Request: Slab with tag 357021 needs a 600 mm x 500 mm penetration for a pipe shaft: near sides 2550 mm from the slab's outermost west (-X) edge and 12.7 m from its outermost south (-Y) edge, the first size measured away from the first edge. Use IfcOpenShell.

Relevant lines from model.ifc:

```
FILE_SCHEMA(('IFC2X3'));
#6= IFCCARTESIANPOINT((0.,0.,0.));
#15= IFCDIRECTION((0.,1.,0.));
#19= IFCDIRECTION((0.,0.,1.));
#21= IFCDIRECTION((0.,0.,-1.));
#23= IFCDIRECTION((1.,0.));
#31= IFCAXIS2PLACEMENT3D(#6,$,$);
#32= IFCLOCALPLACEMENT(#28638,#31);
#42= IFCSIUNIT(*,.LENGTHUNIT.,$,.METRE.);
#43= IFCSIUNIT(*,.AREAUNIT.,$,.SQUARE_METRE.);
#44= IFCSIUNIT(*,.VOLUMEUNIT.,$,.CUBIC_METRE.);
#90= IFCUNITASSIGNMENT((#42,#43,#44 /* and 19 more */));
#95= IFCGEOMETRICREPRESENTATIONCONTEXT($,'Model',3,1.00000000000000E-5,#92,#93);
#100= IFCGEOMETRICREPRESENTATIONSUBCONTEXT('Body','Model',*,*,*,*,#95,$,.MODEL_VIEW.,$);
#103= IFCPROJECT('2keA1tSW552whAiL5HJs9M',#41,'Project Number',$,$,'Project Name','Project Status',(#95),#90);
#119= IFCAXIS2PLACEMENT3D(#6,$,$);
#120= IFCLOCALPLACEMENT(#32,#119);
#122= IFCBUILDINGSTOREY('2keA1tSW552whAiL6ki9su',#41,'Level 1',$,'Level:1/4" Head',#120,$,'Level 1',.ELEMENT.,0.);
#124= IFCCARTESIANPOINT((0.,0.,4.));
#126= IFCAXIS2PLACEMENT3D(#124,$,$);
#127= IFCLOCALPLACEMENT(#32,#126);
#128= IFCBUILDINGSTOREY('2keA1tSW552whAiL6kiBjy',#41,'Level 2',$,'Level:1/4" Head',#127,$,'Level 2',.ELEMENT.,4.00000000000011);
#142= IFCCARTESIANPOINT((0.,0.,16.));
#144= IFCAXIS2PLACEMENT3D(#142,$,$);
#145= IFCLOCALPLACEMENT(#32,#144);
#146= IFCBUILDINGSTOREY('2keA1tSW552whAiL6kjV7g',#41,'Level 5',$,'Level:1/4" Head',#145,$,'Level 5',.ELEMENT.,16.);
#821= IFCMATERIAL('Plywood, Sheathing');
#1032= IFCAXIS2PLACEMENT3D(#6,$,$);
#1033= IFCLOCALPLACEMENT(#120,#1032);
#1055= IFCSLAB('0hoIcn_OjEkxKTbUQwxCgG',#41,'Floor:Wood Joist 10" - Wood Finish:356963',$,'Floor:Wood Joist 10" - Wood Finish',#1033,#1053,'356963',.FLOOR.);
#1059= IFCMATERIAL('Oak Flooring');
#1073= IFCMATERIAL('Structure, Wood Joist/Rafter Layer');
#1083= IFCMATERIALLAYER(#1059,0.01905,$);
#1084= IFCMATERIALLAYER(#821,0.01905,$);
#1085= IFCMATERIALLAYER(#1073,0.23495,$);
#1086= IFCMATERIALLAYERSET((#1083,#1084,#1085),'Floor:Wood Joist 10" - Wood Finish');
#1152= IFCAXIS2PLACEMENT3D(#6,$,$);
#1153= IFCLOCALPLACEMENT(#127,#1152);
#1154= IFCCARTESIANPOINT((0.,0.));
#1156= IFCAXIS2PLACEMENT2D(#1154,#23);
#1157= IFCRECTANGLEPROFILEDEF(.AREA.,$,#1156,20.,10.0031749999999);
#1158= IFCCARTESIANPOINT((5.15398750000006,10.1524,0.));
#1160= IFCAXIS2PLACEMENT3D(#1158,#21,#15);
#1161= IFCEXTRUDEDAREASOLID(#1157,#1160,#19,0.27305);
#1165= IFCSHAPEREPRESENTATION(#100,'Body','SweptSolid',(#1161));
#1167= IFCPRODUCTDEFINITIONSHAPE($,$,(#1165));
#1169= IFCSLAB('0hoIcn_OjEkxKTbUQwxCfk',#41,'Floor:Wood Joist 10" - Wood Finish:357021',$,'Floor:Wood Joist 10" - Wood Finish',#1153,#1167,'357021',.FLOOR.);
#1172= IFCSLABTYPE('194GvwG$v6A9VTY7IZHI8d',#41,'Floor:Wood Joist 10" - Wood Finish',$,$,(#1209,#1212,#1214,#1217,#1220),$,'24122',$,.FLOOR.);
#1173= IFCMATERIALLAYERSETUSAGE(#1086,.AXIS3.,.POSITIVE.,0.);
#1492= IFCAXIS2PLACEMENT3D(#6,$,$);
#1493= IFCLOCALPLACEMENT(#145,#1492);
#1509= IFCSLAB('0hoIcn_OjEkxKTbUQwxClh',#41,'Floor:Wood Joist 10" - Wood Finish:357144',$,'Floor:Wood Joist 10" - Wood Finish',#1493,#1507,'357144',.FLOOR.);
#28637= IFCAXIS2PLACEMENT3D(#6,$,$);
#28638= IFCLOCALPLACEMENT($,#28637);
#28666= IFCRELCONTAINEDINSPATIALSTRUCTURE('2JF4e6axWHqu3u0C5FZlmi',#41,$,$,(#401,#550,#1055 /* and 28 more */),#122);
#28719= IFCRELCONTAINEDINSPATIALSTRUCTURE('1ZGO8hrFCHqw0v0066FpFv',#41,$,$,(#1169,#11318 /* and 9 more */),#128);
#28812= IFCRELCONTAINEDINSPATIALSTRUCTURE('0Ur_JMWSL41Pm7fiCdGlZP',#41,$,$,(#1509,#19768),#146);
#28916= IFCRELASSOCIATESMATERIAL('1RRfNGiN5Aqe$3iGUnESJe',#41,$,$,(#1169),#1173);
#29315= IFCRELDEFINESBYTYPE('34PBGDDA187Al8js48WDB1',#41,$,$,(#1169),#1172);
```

```python
import numpy as np
import ifcopenshell
import ifcopenshell.api.feature
import ifcopenshell.api.geometry
import ifcopenshell.api.root
import ifcopenshell.geom
import ifcopenshell.util.placement
import ifcopenshell.util.representation
import ifcopenshell.util.shape
import ifcopenshell.util.unit

model = ifcopenshell.open("model.ifc")
unit_scale = ifcopenshell.util.unit.calculate_unit_scale(model)
settings = ifcopenshell.geom.settings()


def volume(element):
    """Net volume in cubic metres, openings subtracted."""
    shape = ifcopenshell.geom.create_shape(settings, element)
    return ifcopenshell.util.shape.get_volume(shape.geometry)


slab = model.by_guid("0hoIcn_OjEkxKTbUQwxCfk")
before = volume(slab)

# Extent in the slab's own axes, in metres. The edges named are its -X and -Y sides.
slab_shape = ifcopenshell.geom.create_shape(settings, slab)
vertices = ifcopenshell.util.shape.get_vertices(slab_shape.geometry)
x_min, y_min, bottom = vertices.min(axis=0)
top = vertices[:, 2].max()

opening = ifcopenshell.api.root.create_entity(model, ifc_class="IfcOpeningElement", name="Pipe shaft opening")
context = ifcopenshell.util.representation.get_context(model, "Model", "Body", "MODEL_VIEW")
width, depth = 0.6, 0.5
outline = [(0.0, 0.0), (width, 0.0), (width, depth), (0.0, depth), (0.0, 0.0)]
# Overshoot both faces by 50 mm so the cut is clean.
shape = ifcopenshell.api.geometry.add_slab_representation(
    model, context=context, depth=top - bottom + 0.1, polyline=outline
)
ifcopenshell.api.geometry.assign_representation(model, product=opening, representation=shape)

matrix = ifcopenshell.util.placement.get_local_placement(slab.ObjectPlacement)
matrix[:, 3] = matrix @ np.append(np.array([x_min + 2.55, y_min + 12.7, bottom - 0.05]) / unit_scale, 1.0)
ifcopenshell.api.geometry.edit_object_placement(model, product=opening, matrix=matrix, is_si=False)
ifcopenshell.api.feature.add_feature(model, feature=opening, element=slab)

after = volume(slab)

print(f"slab volume {before:.3f} -> {after:.3f} m3")

model.write("model_v2.ifc")
```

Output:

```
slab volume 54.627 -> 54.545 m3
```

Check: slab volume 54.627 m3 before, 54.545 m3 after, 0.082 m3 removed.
